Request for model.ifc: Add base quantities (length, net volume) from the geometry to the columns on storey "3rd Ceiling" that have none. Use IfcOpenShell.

First a look at what the model holds.

```python
import ifcopenshell
import ifcopenshell.util.element
import ifcopenshell.util.unit

model = ifcopenshell.open("model.ifc")
print(model.schema)
for unit_type in ("LENGTHUNIT", "AREAUNIT", "VOLUMEUNIT"):
    print(unit_type, ifcopenshell.util.unit.calculate_unit_scale(model, unit_type))
storey = next(s for s in model.by_type("IfcBuildingStorey") if s.Name == "3rd Ceiling")
columns = [e for e in ifcopenshell.util.element.get_decomposition(storey) if e.is_a("IfcColumn")]
for e in sorted(columns, key=lambda e: e.id()):
    print(e.id(), e.is_a(), e.Name, list(ifcopenshell.util.element.get_psets(e, qtos_only=True)), sep=" | ")
```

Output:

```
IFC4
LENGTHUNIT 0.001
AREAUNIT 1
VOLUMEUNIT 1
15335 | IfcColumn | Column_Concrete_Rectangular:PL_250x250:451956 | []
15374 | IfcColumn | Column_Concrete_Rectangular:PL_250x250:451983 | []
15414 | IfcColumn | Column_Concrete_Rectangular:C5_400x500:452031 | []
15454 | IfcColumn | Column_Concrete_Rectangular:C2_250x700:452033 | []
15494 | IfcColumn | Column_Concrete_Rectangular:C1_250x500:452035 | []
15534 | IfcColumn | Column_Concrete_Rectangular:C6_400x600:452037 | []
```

```python
import ifcopenshell
import ifcopenshell.api.pset
import ifcopenshell.geom
import ifcopenshell.util.element
import ifcopenshell.util.shape
import ifcopenshell.util.unit

model = ifcopenshell.open("model.ifc")
unit_scale = ifcopenshell.util.unit.calculate_unit_scale(model)
volume_scale = ifcopenshell.util.unit.calculate_unit_scale(model, "VOLUMEUNIT")
settings = ifcopenshell.geom.settings()

storey = next(s for s in model.by_type("IfcBuildingStorey") if s.Name == "3rd Ceiling")
columns = [e for e in ifcopenshell.util.element.get_decomposition(storey) if e.is_a("IfcColumn")]

for e in sorted(columns, key=lambda e: e.id()):
    if ifcopenshell.util.element.get_psets(e, qtos_only=True, should_inherit=False):
        continue
    # Geometry comes back in metres, in the element's own axes.
    shape = ifcopenshell.geom.create_shape(settings, e)
    values = {
        "Length": ifcopenshell.util.shape.get_z(shape.geometry) / unit_scale,
        "NetVolume": ifcopenshell.util.shape.get_volume(shape.geometry) / volume_scale,
    }
    qto = ifcopenshell.api.pset.add_qto(model, product=e, name="Qto_ColumnBaseQuantities")
    ifcopenshell.api.pset.edit_qto(model, qto=qto, properties=values)
    print(e.id(), {k: round(v, 3) for k, v in values.items()})

model.write("model_v2.ifc")
```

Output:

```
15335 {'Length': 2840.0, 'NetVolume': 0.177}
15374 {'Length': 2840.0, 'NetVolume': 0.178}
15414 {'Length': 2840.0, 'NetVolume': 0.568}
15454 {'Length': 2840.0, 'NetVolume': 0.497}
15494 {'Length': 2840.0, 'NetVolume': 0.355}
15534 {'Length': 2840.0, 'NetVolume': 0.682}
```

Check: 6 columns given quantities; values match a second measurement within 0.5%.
